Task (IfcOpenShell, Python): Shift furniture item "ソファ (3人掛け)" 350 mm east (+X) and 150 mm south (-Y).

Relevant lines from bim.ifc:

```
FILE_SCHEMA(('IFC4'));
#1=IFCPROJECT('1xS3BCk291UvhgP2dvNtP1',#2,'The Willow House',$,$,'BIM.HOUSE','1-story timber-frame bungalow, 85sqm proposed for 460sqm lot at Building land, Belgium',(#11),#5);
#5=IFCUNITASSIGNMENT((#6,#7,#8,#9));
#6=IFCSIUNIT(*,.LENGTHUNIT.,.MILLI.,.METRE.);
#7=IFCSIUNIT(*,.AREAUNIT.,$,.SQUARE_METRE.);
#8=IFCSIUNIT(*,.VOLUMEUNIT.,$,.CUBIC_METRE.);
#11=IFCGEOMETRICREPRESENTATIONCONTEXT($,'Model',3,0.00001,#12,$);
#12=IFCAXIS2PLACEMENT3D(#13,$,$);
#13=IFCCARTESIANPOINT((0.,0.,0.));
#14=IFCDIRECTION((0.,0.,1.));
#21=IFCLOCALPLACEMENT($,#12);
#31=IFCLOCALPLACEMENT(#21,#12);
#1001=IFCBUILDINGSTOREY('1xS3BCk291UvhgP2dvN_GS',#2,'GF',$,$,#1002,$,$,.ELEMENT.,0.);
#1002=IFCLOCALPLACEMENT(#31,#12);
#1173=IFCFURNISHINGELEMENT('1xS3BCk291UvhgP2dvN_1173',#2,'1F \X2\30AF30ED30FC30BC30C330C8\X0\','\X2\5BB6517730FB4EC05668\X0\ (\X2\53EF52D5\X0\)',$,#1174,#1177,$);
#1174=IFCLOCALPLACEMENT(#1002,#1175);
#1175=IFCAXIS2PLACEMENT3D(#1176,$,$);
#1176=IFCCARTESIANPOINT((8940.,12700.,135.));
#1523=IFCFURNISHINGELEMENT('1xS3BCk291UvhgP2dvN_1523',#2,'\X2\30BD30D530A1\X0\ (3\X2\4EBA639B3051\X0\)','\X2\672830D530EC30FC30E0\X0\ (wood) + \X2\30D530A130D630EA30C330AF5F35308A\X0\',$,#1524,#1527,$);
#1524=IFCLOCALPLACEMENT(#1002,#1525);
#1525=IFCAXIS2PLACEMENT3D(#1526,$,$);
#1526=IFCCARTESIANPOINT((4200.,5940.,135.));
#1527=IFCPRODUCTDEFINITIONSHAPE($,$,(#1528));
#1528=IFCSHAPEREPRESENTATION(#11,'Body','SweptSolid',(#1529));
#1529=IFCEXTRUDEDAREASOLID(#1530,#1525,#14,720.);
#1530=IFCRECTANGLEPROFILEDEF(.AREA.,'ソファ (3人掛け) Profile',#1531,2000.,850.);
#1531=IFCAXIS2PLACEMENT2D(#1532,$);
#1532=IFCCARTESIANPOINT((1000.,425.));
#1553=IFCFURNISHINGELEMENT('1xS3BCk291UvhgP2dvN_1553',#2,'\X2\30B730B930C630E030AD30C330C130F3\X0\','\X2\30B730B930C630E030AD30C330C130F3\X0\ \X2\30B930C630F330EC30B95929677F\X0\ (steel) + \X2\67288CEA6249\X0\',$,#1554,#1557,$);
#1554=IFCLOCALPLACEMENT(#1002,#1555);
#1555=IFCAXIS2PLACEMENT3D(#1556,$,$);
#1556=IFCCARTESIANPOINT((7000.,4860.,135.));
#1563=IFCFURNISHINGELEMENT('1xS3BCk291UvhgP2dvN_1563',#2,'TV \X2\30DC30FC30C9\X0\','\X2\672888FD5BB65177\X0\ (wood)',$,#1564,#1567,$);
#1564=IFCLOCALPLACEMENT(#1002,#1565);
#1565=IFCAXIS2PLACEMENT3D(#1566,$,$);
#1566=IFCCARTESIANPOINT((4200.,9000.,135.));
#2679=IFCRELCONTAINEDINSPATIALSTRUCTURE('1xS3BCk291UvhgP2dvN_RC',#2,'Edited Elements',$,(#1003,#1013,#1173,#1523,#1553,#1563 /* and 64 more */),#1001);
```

```python
import ifcopenshell
import ifcopenshell.api.geometry
import ifcopenshell.util.placement
import ifcopenshell.util.unit

model = ifcopenshell.open("bim.ifc")
unit_scale = ifcopenshell.util.unit.calculate_unit_scale(model)

item = model.by_guid("1xS3BCk291UvhgP2dvN_1523")
matrix = ifcopenshell.util.placement.get_local_placement(item.ObjectPlacement)
matrix[0, 3] += 0.35 / unit_scale
matrix[1, 3] -= 0.15 / unit_scale
ifcopenshell.api.geometry.edit_object_placement(model, product=item, matrix=matrix, is_si=False)

print(ifcopenshell.util.placement.get_local_placement(item.ObjectPlacement).round(3) + 0.0)

model.write("bim_updated.ifc")
```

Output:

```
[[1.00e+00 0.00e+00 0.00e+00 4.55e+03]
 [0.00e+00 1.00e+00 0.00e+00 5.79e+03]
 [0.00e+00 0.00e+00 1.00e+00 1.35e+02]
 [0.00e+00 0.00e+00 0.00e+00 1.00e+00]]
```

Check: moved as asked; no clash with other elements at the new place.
